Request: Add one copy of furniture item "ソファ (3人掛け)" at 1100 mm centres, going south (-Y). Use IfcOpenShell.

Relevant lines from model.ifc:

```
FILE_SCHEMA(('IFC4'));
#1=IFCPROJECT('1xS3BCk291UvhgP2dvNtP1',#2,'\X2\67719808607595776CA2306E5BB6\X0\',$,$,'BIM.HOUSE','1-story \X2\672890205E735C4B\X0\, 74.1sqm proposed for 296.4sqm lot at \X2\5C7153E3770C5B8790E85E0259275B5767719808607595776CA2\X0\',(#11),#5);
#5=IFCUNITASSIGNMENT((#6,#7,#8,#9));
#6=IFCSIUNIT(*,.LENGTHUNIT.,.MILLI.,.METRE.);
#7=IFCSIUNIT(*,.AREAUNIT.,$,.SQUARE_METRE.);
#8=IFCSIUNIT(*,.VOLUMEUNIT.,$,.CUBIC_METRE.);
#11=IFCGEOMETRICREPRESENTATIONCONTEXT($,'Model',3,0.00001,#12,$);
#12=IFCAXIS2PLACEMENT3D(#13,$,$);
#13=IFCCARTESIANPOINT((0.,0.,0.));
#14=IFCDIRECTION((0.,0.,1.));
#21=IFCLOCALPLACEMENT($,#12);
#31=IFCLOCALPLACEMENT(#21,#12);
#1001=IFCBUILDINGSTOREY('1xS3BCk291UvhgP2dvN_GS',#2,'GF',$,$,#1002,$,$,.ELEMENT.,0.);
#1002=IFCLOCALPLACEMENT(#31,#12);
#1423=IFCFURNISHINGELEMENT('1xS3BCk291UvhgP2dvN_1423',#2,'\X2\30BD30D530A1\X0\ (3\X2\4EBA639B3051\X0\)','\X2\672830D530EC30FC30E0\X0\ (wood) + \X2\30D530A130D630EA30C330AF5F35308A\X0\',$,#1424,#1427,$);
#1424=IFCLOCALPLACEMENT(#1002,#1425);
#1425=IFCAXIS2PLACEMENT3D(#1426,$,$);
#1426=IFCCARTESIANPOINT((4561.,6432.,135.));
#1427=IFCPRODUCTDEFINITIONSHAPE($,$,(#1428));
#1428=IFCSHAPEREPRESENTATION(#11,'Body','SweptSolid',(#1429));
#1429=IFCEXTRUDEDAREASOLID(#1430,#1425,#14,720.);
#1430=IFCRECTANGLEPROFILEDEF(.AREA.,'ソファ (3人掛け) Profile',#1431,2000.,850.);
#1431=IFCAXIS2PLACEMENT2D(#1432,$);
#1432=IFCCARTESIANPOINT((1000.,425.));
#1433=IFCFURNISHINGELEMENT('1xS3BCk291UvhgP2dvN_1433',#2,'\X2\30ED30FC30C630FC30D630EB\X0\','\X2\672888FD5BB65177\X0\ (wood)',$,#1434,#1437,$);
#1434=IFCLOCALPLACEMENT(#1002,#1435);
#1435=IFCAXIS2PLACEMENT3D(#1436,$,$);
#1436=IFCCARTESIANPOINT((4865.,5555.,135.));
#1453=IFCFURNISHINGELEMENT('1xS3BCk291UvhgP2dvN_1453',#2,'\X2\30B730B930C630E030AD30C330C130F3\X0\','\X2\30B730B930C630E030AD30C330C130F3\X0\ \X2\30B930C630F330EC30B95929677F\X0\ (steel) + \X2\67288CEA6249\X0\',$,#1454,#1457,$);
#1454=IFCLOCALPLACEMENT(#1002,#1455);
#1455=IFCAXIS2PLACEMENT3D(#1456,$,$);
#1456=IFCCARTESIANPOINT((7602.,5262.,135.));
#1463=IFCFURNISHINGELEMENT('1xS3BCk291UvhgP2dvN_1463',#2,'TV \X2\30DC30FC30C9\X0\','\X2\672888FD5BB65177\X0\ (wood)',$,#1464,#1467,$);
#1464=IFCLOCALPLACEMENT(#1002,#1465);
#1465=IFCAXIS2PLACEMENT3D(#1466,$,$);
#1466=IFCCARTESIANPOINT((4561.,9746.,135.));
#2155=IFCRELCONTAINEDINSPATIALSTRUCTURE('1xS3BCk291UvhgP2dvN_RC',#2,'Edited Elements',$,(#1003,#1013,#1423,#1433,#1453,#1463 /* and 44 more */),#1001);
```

```python
import numpy as np
import ifcopenshell
import ifcopenshell.api.geometry
import ifcopenshell.api.root
import ifcopenshell.util.element
import ifcopenshell.util.placement

model = ifcopenshell.open("model.ifc")


def reuse_history(source, copy):
    """copy_class also copies each property set's owner history, people and application; keep the originals."""
    for rel in copy.IsDefinedBy:
        if rel.is_a("IfcRelDefinesByProperties") and (history := rel.RelatingPropertyDefinition.OwnerHistory):
            rel.RelatingPropertyDefinition.OwnerHistory = source.OwnerHistory
            ifcopenshell.util.element.remove_deep2(model, history)


source = model.by_id(1423)
base = ifcopenshell.util.placement.get_local_placement(source.ObjectPlacement)
step = np.array([0.0, -1.0, 0.0]) * 1100.0

for i in range(1, 2):
    copy = ifcopenshell.api.root.copy_class(model, product=source)
    copy.Representation = ifcopenshell.util.element.copy_deep(
        model, source.Representation, exclude=["IfcGeometricRepresentationContext", "IfcRepresentationMap"]
    )
    reuse_history(source, copy)
    matrix = base.copy()
    matrix[:3, 3] += i * step
    print("added at", matrix[:3, 3].round(3) + 0.0)
    ifcopenshell.api.geometry.edit_object_placement(model, product=copy, matrix=matrix, is_si=False)

model.write("model_rev.ifc")
```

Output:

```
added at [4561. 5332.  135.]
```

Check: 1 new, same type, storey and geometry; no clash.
